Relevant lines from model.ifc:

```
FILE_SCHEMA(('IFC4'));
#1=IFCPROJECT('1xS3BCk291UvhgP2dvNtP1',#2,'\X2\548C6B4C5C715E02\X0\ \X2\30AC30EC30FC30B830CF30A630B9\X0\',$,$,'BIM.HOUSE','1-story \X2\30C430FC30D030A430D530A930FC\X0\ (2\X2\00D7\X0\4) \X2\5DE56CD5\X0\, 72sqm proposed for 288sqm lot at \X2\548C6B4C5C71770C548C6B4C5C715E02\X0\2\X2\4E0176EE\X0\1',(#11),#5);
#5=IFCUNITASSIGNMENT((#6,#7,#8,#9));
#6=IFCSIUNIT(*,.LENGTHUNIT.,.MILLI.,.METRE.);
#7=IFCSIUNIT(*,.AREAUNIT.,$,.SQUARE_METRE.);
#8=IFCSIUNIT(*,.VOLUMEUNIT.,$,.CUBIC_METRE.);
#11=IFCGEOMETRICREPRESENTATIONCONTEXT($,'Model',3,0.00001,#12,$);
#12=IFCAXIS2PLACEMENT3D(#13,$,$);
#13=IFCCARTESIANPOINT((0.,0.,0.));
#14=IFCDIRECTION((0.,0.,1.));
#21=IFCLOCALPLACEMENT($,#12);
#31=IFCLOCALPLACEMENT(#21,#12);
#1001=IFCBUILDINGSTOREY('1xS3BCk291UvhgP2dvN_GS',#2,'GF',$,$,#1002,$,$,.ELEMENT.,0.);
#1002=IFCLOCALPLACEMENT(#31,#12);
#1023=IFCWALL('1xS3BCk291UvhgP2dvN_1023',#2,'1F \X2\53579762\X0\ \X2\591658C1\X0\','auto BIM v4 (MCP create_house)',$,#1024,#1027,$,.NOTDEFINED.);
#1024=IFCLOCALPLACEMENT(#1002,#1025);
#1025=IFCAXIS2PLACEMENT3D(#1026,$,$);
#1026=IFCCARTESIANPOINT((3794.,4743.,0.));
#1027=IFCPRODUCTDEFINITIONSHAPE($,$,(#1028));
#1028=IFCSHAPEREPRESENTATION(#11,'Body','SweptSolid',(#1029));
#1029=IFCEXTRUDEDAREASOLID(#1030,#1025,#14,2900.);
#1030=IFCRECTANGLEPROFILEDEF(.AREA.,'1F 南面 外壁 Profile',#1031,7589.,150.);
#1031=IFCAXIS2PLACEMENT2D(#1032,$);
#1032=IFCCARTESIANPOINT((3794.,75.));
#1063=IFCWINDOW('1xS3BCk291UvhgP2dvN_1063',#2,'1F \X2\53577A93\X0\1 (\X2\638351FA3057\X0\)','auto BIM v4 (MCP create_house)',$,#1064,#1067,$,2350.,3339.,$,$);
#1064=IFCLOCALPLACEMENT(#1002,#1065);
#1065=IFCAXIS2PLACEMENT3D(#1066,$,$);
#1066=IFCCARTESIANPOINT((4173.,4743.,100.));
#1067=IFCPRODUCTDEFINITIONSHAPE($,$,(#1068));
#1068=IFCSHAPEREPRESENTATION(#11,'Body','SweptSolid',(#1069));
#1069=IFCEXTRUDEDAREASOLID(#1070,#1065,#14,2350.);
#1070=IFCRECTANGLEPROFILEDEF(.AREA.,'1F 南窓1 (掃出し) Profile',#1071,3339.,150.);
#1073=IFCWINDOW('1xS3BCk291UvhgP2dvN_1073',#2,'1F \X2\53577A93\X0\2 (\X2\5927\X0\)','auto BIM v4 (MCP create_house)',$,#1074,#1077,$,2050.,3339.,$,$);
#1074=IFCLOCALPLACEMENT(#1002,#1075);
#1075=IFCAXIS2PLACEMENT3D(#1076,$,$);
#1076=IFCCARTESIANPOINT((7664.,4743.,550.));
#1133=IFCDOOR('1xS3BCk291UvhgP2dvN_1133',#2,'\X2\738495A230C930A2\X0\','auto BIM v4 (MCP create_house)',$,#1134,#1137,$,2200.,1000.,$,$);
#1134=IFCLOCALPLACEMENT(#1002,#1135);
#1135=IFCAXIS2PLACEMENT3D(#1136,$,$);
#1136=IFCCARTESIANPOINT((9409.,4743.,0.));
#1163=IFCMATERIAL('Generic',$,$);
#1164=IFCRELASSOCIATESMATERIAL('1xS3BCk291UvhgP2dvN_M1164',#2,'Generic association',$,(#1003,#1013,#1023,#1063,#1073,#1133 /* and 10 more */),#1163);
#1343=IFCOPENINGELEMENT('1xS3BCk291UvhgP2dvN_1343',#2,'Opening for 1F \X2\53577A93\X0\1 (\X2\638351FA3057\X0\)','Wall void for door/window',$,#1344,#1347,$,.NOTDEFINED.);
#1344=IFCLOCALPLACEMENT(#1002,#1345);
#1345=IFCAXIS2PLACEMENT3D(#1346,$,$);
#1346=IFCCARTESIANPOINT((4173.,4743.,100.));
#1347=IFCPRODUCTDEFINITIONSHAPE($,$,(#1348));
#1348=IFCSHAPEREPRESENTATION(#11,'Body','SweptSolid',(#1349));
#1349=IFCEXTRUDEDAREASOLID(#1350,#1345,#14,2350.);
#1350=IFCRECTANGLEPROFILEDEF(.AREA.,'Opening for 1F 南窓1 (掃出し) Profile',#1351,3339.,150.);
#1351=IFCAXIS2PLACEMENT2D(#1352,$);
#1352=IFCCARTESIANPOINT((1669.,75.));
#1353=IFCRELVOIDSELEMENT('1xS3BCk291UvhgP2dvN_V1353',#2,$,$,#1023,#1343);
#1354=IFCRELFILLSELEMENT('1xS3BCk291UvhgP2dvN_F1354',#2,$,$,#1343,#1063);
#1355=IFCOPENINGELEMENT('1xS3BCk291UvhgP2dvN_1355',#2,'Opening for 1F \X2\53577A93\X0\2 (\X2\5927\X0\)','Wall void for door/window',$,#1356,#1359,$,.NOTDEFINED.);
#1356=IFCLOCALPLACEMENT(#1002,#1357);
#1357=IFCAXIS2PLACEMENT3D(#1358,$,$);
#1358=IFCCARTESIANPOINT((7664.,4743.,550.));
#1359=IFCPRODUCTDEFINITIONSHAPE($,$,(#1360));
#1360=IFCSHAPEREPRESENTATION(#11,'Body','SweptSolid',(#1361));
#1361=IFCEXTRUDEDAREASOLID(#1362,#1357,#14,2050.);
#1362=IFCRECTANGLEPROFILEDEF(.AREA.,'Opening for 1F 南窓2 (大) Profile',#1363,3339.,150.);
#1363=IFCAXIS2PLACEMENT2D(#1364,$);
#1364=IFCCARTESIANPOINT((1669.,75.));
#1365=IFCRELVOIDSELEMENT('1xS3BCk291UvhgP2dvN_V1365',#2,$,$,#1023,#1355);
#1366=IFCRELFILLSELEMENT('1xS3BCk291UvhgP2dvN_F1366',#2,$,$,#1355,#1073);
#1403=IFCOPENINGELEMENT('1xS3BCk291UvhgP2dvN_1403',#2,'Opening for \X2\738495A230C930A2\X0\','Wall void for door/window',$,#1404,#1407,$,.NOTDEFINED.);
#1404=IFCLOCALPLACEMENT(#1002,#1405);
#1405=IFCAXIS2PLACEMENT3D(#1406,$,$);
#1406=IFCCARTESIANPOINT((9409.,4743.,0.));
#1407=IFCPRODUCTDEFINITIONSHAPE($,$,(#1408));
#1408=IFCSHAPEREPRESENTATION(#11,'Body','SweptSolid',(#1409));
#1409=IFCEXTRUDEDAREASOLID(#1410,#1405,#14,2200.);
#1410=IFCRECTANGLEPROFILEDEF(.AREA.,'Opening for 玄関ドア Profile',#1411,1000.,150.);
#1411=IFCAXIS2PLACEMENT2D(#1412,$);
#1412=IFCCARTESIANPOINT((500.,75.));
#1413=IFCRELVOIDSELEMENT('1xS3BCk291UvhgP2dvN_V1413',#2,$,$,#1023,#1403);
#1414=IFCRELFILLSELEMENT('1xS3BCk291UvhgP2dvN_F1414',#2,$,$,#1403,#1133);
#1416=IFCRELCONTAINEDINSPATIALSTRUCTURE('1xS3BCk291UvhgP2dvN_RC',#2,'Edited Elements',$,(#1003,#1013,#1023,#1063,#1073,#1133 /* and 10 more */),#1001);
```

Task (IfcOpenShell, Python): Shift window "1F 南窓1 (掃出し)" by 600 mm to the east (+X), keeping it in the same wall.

```python
import ifcopenshell
import ifcopenshell.api.geometry
import ifcopenshell.util.placement
import ifcopenshell.util.unit

model = ifcopenshell.open("model.ifc")
unit_scale = ifcopenshell.util.unit.calculate_unit_scale(model)

window = model.by_guid("1xS3BCk291UvhgP2dvN_1063")
opening = window.FillsVoids[0].RelatingOpeningElement
wall = opening.VoidsElements[0].RelatingBuildingElement

wall_matrix = ifcopenshell.util.placement.get_local_placement(wall.ObjectPlacement)
shift = wall_matrix[:3, 0] * 0.6 / unit_scale
before = ifcopenshell.util.placement.get_local_placement(window.ObjectPlacement)[:3, 3].copy()

# The window is not placed relative to its opening, so move both.
for product in (opening, window):
    matrix = ifcopenshell.util.placement.get_local_placement(product.ObjectPlacement)
    matrix[:3, 3] += shift
    ifcopenshell.api.geometry.edit_object_placement(model, product=product, matrix=matrix, is_si=False)

after = ifcopenshell.util.placement.get_local_placement(window.ObjectPlacement)[:3, 3]
print("window moved by", (after - before).round(3) + 0.0)

model.write("model_rev.ifc")
```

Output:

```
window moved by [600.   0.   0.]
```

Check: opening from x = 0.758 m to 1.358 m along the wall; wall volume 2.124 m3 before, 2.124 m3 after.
